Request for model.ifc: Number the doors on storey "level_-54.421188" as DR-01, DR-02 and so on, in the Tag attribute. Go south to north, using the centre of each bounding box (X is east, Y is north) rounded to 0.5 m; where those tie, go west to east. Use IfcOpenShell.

First a look at what the model holds.

```python
import ifcopenshell
import ifcopenshell.util.element
import ifcopenshell.util.placement

model = ifcopenshell.open("model.ifc")
print(model.schema)
storey = next(s for s in model.by_type("IfcBuildingStorey") if s.Name == "level_-54.421188")
doors = [e for e in ifcopenshell.util.element.get_decomposition(storey) if e.is_a("IfcDoor")]
for e in sorted(doors, key=lambda e: e.id()):
    origin = ifcopenshell.util.placement.get_local_placement(e.ObjectPlacement)[:3, 3]
    print(e.id(), e.Tag, e.Name, origin.round(2) + 0.0, sep=" | ")
```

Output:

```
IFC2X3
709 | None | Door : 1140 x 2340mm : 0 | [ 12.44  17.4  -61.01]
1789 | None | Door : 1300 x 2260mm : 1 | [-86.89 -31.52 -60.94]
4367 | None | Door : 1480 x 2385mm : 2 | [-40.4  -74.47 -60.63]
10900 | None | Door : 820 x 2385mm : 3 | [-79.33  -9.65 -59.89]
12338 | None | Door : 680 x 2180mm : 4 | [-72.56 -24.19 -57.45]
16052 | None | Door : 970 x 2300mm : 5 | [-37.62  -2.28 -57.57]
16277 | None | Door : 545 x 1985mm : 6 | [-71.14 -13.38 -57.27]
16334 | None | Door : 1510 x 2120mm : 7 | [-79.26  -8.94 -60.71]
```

```python
import ifcopenshell
import ifcopenshell.geom
import ifcopenshell.util.element
import ifcopenshell.util.shape

model = ifcopenshell.open("model.ifc")
settings = ifcopenshell.geom.settings()
settings.set("use-world-coords", True)


def centre(element):
    shape = ifcopenshell.geom.create_shape(settings, element)
    return ifcopenshell.util.shape.get_bbox_centroid(shape.geometry)


storey = next(s for s in model.by_type("IfcBuildingStorey") if s.Name == "level_-54.421188")
doors = [e for e in ifcopenshell.util.element.get_decomposition(storey) if e.is_a("IfcDoor")]

# Insertion points can sit at a corner or the storey origin, so sort by the geometry (in metres).
centres = {e: centre(e) for e in doors}
doors.sort(key=lambda e: (round(centres[e][1] / 0.5), centres[e][0]))

for i, e in enumerate(doors, start=1):
    number = f"DR-{i:02d}"
    e.Tag = number
    print(e.id(), number)

model.write("model_edited.ifc")
```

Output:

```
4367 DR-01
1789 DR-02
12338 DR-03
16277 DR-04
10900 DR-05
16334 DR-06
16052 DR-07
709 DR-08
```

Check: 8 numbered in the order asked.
